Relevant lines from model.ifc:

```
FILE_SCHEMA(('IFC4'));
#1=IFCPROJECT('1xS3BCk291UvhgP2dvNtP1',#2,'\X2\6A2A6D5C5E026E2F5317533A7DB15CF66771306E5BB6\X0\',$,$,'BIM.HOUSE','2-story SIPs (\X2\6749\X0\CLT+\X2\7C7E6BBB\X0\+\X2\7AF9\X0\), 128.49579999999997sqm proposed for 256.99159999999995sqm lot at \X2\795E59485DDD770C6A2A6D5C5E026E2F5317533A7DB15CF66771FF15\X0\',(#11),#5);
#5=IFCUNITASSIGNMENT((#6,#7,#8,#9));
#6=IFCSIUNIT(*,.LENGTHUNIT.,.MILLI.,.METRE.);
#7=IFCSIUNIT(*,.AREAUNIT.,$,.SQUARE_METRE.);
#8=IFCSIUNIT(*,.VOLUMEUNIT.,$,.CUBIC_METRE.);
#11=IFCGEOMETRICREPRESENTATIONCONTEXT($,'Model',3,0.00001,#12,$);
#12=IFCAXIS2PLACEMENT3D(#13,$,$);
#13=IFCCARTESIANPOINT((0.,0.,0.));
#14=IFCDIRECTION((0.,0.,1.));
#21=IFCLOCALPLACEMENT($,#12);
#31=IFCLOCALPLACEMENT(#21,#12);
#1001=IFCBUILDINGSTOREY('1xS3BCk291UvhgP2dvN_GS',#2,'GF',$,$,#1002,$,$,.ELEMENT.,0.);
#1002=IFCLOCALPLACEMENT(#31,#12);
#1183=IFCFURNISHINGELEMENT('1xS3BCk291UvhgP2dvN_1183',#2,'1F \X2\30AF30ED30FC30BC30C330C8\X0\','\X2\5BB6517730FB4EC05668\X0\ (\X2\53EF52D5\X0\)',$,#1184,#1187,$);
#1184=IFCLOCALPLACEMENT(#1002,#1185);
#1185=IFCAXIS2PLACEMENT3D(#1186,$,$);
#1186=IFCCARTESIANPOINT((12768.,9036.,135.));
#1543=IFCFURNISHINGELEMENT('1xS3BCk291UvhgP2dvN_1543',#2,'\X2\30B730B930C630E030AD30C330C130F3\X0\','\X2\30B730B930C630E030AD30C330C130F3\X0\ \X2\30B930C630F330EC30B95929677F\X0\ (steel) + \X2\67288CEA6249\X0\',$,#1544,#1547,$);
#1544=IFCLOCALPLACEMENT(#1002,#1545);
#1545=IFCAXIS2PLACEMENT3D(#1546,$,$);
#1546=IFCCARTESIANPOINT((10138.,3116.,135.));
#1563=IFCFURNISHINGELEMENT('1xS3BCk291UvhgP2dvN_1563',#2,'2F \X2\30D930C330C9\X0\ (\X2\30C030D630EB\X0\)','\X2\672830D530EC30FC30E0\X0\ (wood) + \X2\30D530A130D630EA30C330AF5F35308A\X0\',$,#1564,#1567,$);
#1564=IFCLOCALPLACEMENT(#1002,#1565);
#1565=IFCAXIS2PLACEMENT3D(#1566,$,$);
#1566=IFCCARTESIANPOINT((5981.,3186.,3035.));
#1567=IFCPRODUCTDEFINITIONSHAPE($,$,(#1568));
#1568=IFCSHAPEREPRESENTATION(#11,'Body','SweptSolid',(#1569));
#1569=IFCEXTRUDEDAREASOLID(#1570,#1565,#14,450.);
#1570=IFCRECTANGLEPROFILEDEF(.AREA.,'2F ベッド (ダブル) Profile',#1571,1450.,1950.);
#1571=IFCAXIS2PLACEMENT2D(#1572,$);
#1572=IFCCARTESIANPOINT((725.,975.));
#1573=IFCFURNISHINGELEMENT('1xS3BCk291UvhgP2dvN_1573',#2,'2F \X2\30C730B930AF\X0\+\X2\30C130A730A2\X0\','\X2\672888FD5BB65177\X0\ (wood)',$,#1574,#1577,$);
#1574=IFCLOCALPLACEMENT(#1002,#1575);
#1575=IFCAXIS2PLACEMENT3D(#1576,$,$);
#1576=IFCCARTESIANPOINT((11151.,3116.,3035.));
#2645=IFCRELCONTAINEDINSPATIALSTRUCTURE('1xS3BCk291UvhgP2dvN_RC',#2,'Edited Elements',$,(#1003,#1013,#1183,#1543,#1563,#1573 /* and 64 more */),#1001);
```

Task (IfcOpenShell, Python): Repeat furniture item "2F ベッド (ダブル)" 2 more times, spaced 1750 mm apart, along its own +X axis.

```python
import ifcopenshell
import ifcopenshell.api.geometry
import ifcopenshell.api.root
import ifcopenshell.util.element
import ifcopenshell.util.placement
import ifcopenshell.util.unit

model = ifcopenshell.open("model.ifc")
unit_scale = ifcopenshell.util.unit.calculate_unit_scale(model)


def reuse_history(source, copy):
    """copy_class also copies each property set's owner history, people and application; keep the originals."""
    for rel in copy.IsDefinedBy:
        if rel.is_a("IfcRelDefinesByProperties") and (history := rel.RelatingPropertyDefinition.OwnerHistory):
            rel.RelatingPropertyDefinition.OwnerHistory = source.OwnerHistory
            ifcopenshell.util.element.remove_deep2(model, history)


source = model.by_guid("1xS3BCk291UvhgP2dvN_1563")
base = ifcopenshell.util.placement.get_local_placement(source.ObjectPlacement)
step = base[:3, 0] * 1.75 / unit_scale

for i in range(1, 3):
    copy = ifcopenshell.api.root.copy_class(model, product=source)
    copy.Representation = ifcopenshell.util.element.copy_deep(
        model, source.Representation, exclude=["IfcGeometricRepresentationContext", "IfcRepresentationMap"]
    )
    reuse_history(source, copy)
    matrix = base.copy()
    matrix[:3, 3] += i * step
    print("added at", matrix[:3, 3].round(3) + 0.0)
    ifcopenshell.api.geometry.edit_object_placement(model, product=copy, matrix=matrix, is_si=False)

model.write("model_updated.ifc")
```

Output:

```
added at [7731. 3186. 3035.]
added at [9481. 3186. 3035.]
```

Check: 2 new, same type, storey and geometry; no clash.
